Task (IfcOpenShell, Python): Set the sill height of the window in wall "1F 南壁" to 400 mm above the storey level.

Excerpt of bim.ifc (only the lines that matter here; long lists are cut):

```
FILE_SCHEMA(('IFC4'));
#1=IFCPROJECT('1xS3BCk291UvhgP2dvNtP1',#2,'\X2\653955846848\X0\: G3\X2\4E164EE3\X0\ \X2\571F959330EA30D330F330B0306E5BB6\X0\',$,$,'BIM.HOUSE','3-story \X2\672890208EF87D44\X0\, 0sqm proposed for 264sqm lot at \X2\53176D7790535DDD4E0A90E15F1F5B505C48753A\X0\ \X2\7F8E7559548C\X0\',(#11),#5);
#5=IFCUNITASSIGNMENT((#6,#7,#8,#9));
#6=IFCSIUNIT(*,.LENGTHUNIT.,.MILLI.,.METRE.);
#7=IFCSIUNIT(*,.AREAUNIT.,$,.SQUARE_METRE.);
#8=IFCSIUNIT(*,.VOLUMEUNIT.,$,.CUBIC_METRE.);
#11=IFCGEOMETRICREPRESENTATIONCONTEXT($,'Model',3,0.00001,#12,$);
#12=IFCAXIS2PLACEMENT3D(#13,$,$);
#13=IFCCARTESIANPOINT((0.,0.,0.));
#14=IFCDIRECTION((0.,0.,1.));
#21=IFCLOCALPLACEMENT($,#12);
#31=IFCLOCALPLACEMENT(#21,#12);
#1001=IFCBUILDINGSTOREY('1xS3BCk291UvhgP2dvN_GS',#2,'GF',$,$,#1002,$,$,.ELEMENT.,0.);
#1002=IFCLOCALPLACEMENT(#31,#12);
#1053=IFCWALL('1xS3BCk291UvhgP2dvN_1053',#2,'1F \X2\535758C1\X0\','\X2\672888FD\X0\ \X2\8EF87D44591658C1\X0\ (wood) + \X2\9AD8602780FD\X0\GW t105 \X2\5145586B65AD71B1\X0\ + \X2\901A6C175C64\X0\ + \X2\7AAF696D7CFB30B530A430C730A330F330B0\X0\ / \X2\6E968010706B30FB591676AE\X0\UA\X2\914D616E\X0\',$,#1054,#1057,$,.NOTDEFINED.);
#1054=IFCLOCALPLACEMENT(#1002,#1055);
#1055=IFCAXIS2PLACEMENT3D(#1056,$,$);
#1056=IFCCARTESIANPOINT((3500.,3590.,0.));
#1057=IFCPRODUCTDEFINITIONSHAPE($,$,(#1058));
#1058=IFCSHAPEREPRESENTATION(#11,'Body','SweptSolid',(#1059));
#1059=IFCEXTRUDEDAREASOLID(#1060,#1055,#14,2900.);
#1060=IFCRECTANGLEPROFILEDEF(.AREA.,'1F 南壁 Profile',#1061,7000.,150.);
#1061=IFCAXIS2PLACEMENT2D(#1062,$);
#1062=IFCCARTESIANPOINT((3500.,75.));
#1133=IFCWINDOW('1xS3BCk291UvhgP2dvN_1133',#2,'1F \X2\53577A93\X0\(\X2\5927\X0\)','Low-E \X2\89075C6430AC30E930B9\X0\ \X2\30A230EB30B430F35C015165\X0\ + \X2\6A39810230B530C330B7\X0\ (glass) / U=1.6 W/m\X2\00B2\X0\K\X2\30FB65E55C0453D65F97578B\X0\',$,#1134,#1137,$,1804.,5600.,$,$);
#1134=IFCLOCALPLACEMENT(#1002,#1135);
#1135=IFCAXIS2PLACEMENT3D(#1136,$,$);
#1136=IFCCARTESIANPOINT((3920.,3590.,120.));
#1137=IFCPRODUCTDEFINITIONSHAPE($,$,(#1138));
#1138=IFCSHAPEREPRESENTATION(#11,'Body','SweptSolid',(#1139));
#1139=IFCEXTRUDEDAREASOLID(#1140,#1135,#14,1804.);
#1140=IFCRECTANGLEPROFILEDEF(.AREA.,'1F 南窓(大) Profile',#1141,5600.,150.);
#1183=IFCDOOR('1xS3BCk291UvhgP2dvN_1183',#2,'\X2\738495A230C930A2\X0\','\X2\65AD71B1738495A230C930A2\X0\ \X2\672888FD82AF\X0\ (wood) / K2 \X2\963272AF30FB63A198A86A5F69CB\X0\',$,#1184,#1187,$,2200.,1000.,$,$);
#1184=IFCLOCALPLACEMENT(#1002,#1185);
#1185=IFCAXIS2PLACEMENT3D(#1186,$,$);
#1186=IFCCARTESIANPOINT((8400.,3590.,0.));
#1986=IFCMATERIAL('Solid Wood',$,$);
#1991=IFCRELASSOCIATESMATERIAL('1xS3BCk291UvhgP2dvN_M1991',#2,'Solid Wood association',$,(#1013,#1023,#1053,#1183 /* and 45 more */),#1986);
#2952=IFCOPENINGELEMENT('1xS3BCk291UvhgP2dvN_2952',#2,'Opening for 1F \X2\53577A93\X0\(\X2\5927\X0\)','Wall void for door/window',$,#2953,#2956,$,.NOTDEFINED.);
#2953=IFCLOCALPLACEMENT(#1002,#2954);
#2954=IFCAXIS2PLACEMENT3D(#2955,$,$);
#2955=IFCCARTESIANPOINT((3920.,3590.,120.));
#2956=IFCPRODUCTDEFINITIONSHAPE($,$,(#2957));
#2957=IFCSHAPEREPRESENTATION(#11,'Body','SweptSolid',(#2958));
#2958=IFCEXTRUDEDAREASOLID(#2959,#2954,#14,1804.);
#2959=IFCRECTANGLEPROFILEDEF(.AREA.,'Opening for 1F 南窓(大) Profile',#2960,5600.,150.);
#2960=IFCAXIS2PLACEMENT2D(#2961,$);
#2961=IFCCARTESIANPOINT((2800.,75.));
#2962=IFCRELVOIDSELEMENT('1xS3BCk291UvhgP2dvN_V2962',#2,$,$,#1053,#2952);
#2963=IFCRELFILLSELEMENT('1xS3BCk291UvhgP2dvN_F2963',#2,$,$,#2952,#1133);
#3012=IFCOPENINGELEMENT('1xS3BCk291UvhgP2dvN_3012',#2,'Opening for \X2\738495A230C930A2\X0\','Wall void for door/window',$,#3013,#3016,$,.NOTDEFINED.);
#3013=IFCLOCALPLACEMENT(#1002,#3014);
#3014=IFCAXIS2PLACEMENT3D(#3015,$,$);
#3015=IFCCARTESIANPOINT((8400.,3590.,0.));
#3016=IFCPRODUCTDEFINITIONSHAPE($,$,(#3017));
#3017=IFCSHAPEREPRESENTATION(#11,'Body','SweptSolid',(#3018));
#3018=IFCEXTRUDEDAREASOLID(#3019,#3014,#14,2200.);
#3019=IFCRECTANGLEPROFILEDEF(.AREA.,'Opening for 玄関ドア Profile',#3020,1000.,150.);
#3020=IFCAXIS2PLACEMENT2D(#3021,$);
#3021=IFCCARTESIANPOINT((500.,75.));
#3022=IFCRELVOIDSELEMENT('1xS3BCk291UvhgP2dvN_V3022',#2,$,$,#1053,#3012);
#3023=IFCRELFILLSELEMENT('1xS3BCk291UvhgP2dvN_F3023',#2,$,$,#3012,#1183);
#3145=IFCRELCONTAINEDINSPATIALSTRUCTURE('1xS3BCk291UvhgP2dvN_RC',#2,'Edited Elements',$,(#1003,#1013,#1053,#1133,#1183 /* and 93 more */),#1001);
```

```python
import numpy as np
import ifcopenshell
import ifcopenshell.api.geometry
import ifcopenshell.geom
import ifcopenshell.util.element
import ifcopenshell.util.placement
import ifcopenshell.util.shape
import ifcopenshell.util.unit

model = ifcopenshell.open("bim.ifc")
unit_scale = ifcopenshell.util.unit.calculate_unit_scale(model)

window = model.by_guid("1xS3BCk291UvhgP2dvN_1133")
opening = window.FillsVoids[0].RelatingOpeningElement
storey = ifcopenshell.util.element.get_container(window, ifc_class="IfcBuildingStorey")
level = ifcopenshell.util.placement.get_local_placement(storey.ObjectPlacement)[2, 3]

# The opening's origin need not be at the sill, so measure its lowest point.
shape = ifcopenshell.geom.create_shape(ifcopenshell.geom.settings(), opening)
bottom = ifcopenshell.util.shape.get_shape_bottom_elevation(shape, shape.geometry) / unit_scale
dz = level + 400.0 - bottom

shift = np.array([0.0, 0.0, dz])
# The window is not placed relative to its opening, so move both.
for product in (opening, window):
    matrix = ifcopenshell.util.placement.get_local_placement(product.ObjectPlacement)
    matrix[:3, 3] += shift
    ifcopenshell.api.geometry.edit_object_placement(model, product=product, matrix=matrix, is_si=False)

print(f"moved by {dz * unit_scale:+.3f} m")

model.write("bim_edited.ifc")
```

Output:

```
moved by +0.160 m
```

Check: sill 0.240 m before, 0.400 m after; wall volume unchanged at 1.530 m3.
